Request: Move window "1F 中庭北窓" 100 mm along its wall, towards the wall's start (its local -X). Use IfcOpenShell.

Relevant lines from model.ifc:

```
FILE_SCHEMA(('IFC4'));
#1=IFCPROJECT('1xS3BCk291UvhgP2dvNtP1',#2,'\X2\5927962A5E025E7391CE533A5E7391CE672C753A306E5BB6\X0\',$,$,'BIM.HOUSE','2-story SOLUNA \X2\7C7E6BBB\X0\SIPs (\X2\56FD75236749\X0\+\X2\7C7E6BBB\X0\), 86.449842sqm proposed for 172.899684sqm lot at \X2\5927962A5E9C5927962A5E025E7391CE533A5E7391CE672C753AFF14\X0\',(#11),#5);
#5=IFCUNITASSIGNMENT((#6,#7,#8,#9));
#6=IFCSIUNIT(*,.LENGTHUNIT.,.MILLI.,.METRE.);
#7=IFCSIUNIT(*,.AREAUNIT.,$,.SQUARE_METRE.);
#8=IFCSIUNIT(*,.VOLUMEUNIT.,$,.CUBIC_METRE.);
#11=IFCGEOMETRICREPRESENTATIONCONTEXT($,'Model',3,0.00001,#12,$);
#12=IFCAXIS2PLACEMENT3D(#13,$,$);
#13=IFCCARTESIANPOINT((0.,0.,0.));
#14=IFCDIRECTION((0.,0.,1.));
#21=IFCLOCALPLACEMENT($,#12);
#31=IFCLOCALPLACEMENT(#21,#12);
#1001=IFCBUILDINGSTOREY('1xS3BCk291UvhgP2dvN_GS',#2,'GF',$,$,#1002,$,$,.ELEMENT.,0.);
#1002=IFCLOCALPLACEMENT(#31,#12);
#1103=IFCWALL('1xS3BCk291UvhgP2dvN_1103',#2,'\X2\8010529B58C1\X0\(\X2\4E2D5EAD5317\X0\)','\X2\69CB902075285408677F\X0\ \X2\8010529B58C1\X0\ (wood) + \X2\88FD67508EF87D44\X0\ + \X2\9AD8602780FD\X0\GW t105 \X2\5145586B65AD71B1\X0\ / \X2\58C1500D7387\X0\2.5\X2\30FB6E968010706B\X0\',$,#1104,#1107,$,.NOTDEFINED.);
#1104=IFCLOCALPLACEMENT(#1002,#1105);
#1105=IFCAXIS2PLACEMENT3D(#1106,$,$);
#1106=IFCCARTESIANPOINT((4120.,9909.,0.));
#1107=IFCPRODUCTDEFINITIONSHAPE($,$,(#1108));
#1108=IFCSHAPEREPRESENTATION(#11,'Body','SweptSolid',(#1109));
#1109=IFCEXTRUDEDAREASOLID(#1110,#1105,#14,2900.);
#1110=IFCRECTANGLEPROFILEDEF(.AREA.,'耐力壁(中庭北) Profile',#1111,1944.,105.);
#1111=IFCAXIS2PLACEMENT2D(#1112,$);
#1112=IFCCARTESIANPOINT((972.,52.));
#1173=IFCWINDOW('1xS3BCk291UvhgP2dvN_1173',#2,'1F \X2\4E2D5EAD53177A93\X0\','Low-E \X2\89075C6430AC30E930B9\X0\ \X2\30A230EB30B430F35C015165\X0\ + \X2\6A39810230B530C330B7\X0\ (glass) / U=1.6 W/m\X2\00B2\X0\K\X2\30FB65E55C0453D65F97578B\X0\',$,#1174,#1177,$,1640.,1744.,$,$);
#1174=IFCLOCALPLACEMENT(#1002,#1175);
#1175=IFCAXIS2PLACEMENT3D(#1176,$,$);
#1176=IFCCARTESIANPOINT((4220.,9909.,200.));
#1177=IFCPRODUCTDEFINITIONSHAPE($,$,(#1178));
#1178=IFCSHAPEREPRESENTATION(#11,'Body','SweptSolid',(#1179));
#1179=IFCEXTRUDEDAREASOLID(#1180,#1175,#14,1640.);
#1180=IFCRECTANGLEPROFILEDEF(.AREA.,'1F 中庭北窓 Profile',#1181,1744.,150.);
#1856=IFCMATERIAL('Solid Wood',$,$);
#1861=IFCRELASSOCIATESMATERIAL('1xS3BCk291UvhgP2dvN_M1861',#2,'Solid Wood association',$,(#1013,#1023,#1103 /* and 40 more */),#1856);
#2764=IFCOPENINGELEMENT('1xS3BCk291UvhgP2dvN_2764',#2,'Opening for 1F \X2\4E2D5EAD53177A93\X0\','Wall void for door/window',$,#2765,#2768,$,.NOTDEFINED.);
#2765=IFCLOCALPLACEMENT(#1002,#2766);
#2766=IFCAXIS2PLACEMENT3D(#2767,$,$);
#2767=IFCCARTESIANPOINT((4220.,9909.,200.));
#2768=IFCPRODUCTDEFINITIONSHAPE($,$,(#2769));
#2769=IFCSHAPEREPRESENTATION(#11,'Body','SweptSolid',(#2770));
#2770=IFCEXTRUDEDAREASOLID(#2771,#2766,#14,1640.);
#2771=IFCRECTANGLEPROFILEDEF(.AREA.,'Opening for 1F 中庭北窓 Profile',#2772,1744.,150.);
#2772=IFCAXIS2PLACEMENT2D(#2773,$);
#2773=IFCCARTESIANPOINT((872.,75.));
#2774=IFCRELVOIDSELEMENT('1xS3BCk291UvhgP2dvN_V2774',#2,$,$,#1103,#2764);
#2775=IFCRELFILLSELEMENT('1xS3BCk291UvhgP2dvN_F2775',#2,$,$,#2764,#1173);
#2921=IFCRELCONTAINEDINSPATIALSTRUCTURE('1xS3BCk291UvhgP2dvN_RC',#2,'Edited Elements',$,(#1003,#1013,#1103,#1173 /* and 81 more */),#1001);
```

```python
import ifcopenshell
import ifcopenshell.api.geometry
import ifcopenshell.util.placement

model = ifcopenshell.open("model.ifc")

window = model.by_guid("1xS3BCk291UvhgP2dvN_1173")
opening = window.FillsVoids[0].RelatingOpeningElement
wall = opening.VoidsElements[0].RelatingBuildingElement

wall_matrix = ifcopenshell.util.placement.get_local_placement(wall.ObjectPlacement)
shift = wall_matrix[:3, 0] * -100.0
before = ifcopenshell.util.placement.get_local_placement(window.ObjectPlacement)[:3, 3].copy()

# The window is not placed relative to its opening, so move both.
for product in (opening, window):
    matrix = ifcopenshell.util.placement.get_local_placement(product.ObjectPlacement)
    matrix[:3, 3] += shift
    ifcopenshell.api.geometry.edit_object_placement(model, product=product, matrix=matrix, is_si=False)

after = ifcopenshell.util.placement.get_local_placement(window.ObjectPlacement)[:3, 3]
print("window moved by", (after - before).round(3) + 0.0)

model.write("model_updated.ifc")
```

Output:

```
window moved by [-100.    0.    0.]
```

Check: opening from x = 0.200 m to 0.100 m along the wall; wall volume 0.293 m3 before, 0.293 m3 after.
